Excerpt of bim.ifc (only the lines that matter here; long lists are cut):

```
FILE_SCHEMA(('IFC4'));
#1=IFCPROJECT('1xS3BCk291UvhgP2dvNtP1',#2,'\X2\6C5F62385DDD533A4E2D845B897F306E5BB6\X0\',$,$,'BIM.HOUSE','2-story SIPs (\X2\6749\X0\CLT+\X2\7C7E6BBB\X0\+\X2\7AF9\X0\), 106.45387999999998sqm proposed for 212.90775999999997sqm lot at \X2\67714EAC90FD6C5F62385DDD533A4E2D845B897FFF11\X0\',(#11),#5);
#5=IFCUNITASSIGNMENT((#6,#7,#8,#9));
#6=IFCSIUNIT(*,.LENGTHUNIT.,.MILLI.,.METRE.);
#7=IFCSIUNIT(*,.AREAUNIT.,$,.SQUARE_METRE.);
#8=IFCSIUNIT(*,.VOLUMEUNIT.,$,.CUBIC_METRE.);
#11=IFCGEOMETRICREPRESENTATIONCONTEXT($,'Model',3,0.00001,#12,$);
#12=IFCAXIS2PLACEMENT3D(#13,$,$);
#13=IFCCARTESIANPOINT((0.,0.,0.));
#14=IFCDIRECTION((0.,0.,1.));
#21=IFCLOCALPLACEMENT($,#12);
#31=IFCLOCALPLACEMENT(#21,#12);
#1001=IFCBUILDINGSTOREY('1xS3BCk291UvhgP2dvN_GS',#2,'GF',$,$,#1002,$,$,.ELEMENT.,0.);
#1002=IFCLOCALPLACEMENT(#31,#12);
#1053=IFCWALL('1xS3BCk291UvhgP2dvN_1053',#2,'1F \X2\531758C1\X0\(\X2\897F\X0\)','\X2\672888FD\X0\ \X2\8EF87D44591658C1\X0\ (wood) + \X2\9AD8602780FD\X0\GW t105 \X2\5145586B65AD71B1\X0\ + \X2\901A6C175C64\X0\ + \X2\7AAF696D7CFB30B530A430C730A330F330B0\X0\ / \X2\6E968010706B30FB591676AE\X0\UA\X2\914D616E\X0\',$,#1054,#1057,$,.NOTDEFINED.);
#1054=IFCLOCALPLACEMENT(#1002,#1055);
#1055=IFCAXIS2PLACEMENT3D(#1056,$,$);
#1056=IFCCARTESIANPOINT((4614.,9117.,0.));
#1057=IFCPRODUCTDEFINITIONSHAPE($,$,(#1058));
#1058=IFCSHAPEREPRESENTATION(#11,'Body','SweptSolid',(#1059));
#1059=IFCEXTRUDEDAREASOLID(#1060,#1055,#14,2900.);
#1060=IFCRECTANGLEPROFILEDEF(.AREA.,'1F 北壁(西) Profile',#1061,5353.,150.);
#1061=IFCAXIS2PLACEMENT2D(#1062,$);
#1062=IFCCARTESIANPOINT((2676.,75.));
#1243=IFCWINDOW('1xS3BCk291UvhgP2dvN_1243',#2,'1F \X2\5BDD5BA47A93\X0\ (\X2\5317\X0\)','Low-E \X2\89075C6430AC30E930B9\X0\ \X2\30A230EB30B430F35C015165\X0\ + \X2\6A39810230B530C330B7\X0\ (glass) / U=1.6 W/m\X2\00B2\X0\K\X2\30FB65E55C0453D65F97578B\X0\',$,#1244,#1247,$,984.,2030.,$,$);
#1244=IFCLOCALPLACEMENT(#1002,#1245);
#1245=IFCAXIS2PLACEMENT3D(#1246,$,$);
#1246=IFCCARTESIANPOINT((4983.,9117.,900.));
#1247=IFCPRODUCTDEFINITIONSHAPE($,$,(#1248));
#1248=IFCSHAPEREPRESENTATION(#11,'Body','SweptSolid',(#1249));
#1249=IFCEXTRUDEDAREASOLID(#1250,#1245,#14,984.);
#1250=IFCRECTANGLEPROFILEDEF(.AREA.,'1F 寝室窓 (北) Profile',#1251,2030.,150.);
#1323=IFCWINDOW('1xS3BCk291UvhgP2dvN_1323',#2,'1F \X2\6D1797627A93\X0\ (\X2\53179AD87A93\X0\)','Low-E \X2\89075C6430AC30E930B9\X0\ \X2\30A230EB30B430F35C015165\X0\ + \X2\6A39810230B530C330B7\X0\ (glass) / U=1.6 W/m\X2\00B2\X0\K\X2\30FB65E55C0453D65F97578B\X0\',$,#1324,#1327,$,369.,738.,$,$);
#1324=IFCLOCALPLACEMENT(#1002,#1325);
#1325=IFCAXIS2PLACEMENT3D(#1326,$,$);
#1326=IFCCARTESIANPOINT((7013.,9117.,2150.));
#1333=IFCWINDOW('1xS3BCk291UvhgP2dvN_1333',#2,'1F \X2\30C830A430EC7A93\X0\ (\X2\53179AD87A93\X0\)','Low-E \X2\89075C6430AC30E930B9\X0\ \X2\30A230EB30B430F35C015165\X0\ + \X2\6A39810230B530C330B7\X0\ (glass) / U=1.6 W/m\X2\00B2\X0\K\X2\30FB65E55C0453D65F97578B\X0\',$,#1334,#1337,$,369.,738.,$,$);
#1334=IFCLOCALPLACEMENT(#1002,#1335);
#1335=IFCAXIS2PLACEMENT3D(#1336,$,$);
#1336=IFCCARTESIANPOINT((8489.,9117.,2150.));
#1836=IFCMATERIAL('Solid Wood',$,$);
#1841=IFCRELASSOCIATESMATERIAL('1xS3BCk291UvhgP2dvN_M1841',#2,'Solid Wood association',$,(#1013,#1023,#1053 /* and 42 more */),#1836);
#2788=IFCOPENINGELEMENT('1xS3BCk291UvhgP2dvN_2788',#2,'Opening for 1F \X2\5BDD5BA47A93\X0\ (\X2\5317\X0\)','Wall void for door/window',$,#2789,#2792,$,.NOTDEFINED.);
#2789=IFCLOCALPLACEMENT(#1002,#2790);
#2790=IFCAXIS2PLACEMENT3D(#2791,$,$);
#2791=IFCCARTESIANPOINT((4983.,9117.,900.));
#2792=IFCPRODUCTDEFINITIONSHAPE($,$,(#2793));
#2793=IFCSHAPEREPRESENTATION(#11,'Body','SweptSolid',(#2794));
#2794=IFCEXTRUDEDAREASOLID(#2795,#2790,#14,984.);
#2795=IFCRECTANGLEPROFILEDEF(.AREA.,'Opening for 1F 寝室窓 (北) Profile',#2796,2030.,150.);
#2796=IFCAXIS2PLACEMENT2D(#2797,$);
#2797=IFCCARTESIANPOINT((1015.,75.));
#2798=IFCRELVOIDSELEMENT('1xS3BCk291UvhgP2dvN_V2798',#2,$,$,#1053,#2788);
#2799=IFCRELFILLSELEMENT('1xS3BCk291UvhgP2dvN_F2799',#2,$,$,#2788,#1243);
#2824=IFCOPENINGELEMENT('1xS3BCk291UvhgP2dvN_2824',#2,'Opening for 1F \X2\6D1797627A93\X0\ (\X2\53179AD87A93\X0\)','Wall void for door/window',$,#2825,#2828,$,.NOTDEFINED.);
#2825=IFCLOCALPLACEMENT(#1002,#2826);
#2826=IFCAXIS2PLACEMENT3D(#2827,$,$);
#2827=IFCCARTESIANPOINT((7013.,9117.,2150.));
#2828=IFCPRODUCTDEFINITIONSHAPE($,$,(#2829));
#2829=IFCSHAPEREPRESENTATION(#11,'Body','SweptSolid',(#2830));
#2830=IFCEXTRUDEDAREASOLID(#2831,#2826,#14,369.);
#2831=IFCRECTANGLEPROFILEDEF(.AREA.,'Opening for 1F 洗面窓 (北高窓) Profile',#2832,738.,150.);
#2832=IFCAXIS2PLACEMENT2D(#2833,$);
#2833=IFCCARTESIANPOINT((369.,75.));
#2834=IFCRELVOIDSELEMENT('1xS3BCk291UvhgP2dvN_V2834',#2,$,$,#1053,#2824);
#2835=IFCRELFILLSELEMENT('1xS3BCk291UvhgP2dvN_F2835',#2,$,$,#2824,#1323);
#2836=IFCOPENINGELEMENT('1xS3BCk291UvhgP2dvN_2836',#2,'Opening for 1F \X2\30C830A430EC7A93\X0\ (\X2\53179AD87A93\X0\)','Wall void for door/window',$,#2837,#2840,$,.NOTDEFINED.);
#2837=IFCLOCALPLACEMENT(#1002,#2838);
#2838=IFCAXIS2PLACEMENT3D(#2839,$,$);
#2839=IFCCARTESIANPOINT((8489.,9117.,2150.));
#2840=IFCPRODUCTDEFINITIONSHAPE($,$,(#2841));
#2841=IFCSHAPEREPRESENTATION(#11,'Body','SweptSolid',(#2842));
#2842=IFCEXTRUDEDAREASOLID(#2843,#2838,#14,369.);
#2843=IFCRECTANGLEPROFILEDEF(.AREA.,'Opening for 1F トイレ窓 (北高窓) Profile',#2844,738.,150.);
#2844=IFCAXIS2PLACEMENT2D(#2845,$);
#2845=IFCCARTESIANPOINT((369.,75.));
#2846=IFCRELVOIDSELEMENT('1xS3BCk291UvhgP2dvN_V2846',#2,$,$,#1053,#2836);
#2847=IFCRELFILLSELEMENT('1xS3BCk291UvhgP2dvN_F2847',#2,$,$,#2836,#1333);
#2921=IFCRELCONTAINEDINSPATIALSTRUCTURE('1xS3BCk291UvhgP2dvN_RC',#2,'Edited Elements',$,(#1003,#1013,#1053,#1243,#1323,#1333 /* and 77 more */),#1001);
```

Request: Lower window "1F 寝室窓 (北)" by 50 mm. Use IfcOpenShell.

```python
import numpy as np
import ifcopenshell
import ifcopenshell.api.geometry
import ifcopenshell.util.placement
import ifcopenshell.util.unit

model = ifcopenshell.open("bim.ifc")
unit_scale = ifcopenshell.util.unit.calculate_unit_scale(model)

window = model.by_guid("1xS3BCk291UvhgP2dvN_1243")
opening = window.FillsVoids[0].RelatingOpeningElement
dz = -0.05 / unit_scale

shift = np.array([0.0, 0.0, dz])
# The window is not placed relative to its opening, so move both.
for product in (opening, window):
    matrix = ifcopenshell.util.placement.get_local_placement(product.ObjectPlacement)
    matrix[:3, 3] += shift
    ifcopenshell.api.geometry.edit_object_placement(model, product=product, matrix=matrix, is_si=False)

print(f"moved by {dz * unit_scale:+.3f} m")

model.write("bim_rev.ifc")
```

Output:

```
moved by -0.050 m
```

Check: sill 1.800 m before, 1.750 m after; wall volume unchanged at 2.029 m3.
